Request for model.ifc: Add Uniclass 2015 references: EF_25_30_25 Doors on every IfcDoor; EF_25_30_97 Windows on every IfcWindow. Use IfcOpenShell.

First a look at what the model holds.

```python
import ifcopenshell

model = ifcopenshell.open("model.ifc")
print(model.schema)
print("classifications:", [c.Name for c in model.by_type("IfcClassification")])
for ifc_class in ("IfcDoor", "IfcRoof", "IfcStair", "IfcWall", "IfcWindow"):
    print(ifc_class, len(model.by_type(ifc_class)))
```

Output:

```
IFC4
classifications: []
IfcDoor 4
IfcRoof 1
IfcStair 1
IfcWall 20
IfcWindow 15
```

```python
import ifcopenshell
import ifcopenshell.api.classification

model = ifcopenshell.open("model.ifc")

system = ifcopenshell.api.classification.add_classification(model, classification="Uniclass 2015")

codes = {
    "IfcDoor": ("EF_25_30_25", "Doors"),
    "IfcWindow": ("EF_25_30_97", "Windows"),
}
for ifc_class, (code, name) in codes.items():
    products = model.by_type(ifc_class)
    ifcopenshell.api.classification.add_reference(
        model, products=products, classification=system, identification=code, name=name
    )
    print(code, len(products))

model.write("model_updated.ifc")
```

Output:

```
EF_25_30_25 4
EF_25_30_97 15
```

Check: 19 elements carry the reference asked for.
